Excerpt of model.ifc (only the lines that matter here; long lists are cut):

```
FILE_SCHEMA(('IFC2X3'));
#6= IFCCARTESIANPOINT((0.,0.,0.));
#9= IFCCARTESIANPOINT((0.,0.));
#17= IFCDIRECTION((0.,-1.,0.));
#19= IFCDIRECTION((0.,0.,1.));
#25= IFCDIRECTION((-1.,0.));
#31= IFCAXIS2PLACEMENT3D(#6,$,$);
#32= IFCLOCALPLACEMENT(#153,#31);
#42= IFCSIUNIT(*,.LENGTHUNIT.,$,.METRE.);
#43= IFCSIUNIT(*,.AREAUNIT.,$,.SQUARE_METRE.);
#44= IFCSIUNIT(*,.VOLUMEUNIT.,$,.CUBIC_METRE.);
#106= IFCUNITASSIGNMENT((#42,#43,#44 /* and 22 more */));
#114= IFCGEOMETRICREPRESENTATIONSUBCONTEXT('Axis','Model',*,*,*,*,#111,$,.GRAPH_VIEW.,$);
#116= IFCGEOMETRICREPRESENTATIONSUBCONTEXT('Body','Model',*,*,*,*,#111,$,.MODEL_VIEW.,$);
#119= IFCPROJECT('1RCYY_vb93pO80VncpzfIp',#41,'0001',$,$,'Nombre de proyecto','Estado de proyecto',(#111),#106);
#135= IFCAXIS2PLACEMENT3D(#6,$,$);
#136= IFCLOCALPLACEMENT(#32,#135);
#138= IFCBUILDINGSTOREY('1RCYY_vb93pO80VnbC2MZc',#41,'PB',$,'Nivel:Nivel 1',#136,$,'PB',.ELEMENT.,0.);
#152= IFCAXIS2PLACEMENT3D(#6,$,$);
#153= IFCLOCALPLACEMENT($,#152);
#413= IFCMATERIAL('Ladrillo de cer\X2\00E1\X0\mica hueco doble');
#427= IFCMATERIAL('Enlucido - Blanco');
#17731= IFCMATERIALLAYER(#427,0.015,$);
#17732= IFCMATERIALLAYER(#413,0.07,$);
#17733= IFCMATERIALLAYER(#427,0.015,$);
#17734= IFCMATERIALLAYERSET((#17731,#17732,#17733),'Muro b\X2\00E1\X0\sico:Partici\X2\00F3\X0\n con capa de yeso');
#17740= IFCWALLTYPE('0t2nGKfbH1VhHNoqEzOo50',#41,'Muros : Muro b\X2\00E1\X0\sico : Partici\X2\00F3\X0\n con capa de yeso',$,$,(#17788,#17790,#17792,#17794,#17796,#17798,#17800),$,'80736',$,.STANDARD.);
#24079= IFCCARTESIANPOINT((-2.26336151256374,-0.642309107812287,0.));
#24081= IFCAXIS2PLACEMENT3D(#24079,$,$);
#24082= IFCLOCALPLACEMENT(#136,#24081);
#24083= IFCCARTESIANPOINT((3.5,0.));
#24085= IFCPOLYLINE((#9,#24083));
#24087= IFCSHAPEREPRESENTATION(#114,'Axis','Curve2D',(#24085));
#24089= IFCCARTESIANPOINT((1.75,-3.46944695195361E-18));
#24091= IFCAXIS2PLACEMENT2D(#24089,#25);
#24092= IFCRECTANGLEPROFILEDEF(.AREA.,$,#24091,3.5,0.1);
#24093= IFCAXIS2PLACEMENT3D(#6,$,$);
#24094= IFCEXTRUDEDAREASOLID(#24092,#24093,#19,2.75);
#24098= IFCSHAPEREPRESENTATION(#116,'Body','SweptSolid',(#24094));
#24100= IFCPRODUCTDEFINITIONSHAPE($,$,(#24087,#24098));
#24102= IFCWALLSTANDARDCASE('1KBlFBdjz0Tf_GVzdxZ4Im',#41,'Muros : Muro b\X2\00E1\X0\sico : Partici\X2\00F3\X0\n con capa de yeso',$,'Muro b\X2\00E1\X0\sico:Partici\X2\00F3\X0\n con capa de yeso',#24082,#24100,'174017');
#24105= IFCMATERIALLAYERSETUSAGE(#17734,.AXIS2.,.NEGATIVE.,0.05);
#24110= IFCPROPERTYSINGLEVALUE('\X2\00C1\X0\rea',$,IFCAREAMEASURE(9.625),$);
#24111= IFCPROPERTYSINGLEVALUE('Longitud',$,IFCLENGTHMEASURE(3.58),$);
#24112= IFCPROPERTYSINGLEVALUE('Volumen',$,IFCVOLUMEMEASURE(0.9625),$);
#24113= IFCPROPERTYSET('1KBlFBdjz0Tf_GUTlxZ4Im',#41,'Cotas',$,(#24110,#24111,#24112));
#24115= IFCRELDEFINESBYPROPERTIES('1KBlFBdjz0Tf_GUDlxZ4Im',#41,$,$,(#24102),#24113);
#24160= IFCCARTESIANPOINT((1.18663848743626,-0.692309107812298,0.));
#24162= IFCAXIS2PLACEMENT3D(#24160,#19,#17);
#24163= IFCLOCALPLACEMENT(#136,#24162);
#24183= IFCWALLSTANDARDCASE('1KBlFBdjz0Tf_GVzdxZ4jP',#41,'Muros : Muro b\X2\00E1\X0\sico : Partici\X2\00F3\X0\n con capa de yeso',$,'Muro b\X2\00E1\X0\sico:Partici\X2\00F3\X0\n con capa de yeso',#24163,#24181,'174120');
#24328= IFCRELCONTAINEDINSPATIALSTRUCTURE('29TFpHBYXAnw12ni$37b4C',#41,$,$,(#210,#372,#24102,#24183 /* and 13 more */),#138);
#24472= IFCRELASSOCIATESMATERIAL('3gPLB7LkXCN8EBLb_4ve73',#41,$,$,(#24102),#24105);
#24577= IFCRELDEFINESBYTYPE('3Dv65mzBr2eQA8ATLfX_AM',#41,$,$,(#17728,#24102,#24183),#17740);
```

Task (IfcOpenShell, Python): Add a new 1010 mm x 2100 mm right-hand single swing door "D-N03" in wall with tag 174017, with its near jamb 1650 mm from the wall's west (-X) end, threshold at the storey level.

```python
import numpy as np
import ifcopenshell
import ifcopenshell.api.feature
import ifcopenshell.api.geometry
import ifcopenshell.api.pset
import ifcopenshell.api.root
import ifcopenshell.api.spatial
import ifcopenshell.api.type
import ifcopenshell.geom
import ifcopenshell.util.element
import ifcopenshell.util.placement
import ifcopenshell.util.representation
import ifcopenshell.util.shape
import ifcopenshell.util.unit

model = ifcopenshell.open("model.ifc")
unit_scale = ifcopenshell.util.unit.calculate_unit_scale(model)
area_scale = ifcopenshell.util.unit.calculate_unit_scale(model, "AREAUNIT")
volume_scale = ifcopenshell.util.unit.calculate_unit_scale(model, "VOLUMEUNIT")
settings = ifcopenshell.geom.settings()


def volume(element):
    """Net volume in cubic metres, openings subtracted."""
    shape = ifcopenshell.geom.create_shape(settings, element)
    return ifcopenshell.util.shape.get_volume(shape.geometry)


wall = model.by_id(24102)
storey = ifcopenshell.util.element.get_container(wall, ifc_class="IfcBuildingStorey")
context = ifcopenshell.util.representation.get_context(model, "Model", "Body", "MODEL_VIEW")
before = volume(wall)

width, height, from_end, sill = 1.01, 2.1, 1.65, 0.0  # metres

# The wall runs along its own X axis, and the end named is its -X end.
wall_shape = ifcopenshell.geom.create_shape(settings, wall)
x, y, z = ifcopenshell.util.shape.get_vertices(wall_shape.geometry).T
start = x.min() + from_end
face, thickness = float(y.min()), float(y.max() - y.min())
wall_matrix = ifcopenshell.util.placement.get_local_placement(wall.ObjectPlacement)
level = ifcopenshell.util.placement.get_local_placement(storey.ObjectPlacement)[2, 3]


def in_wall(x, y):
    """Placement at x, y metres in the wall's axes, at sill height."""
    matrix = wall_matrix.copy()
    matrix[:, 3] = wall_matrix @ np.array([x / unit_scale, y / unit_scale, 0.0, 1.0])
    matrix[2, 3] = level + sill / unit_scale
    return matrix


# Opening: a box that overshoots both wall faces by 50 mm.
opening = ifcopenshell.api.root.create_entity(model, ifc_class="IfcOpeningElement")
box = ifcopenshell.api.geometry.add_wall_representation(
    model, context=context, length=width, height=height, thickness=thickness + 0.1
)
ifcopenshell.api.geometry.assign_representation(model, product=opening, representation=box)
ifcopenshell.api.geometry.edit_object_placement(model, product=opening, matrix=in_wall(start, face - 0.05), is_si=False)
ifcopenshell.api.feature.add_feature(model, feature=opening, element=wall)

door = ifcopenshell.api.root.create_entity(model, ifc_class="IfcDoor", name="D-N03")
door.OverallWidth, door.OverallHeight = width / unit_scale, height / unit_scale
body = ifcopenshell.api.geometry.add_door_representation(
    model,
    context=context,
    overall_width=door.OverallWidth,
    overall_height=door.OverallHeight,
    operation_type="SINGLE_SWING_RIGHT",
    lining_properties={"LiningDepth": thickness / unit_scale, "ThresholdDepth": thickness / unit_scale},
)
ifcopenshell.api.geometry.assign_representation(model, product=door, representation=body)
ifcopenshell.api.spatial.assign_container(model, products=[door], relating_structure=storey)
fills = ifcopenshell.api.feature.add_filling(model, opening=opening, element=door)
fills.OwnerHistory = door.OwnerHistory  # required in IFC2X3

# IFC2X3 keeps the operation on the door style.
style = ifcopenshell.api.root.create_entity(model, ifc_class="IfcDoorStyle", name="D-N03")
style.OperationType, style.ConstructionType = "SINGLE_SWING_RIGHT", "NOTDEFINED"
style.ParameterTakesPrecedence = style.Sizeable = False
ifcopenshell.api.type.assign_type(model, related_objects=[door], relating_type=style)

# The lining spans the wall, so the door starts at the wall face.
ifcopenshell.api.geometry.edit_object_placement(model, product=door, matrix=in_wall(start, face), is_si=False)

after = volume(wall)

# Update the wall's stored quantities.
pset = model.by_id(ifcopenshell.util.element.get_pset(wall, "Cotas", should_inherit=False)["id"])
ifcopenshell.api.pset.edit_pset(model, pset=pset, properties={
    "Área": model.create_entity("IfcAreaMeasure", after / thickness / area_scale),
    "Volumen": model.create_entity("IfcVolumeMeasure", after / volume_scale),
})

print(f"wall volume {before:.3f} -> {after:.3f} m3")

model.write("model_v2.ifc")
```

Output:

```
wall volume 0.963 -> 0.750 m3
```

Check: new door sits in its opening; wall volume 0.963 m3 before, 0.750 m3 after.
